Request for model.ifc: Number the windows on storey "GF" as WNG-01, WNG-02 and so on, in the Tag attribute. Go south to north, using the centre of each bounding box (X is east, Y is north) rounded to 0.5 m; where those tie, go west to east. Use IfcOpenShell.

First a look at what the model holds.

```python
import ifcopenshell
import ifcopenshell.util.element
import ifcopenshell.util.placement

model = ifcopenshell.open("model.ifc")
print(model.schema)
storey = next(s for s in model.by_type("IfcBuildingStorey") if s.Name == "GF")
windows = [e for e in ifcopenshell.util.element.get_decomposition(storey) if e.is_a("IfcWindow")]
for e in sorted(windows, key=lambda e: e.id()):
    origin = ifcopenshell.util.placement.get_local_placement(e.ObjectPlacement)[:3, 3]
    print(e.id(), e.Tag, e.Name, origin.round(2) + 0.0, sep=" | ")
```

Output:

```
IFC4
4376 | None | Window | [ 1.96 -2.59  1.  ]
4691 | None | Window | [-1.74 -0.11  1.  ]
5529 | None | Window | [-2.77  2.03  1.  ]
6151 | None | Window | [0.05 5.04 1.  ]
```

```python
import ifcopenshell
import ifcopenshell.geom
import ifcopenshell.util.element
import ifcopenshell.util.shape

model = ifcopenshell.open("model.ifc")
settings = ifcopenshell.geom.settings()
settings.set("use-world-coords", True)


def centre(element):
    shape = ifcopenshell.geom.create_shape(settings, element)
    return ifcopenshell.util.shape.get_bbox_centroid(shape.geometry)


storey = next(s for s in model.by_type("IfcBuildingStorey") if s.Name == "GF")
windows = [e for e in ifcopenshell.util.element.get_decomposition(storey) if e.is_a("IfcWindow")]

# Insertion points can sit at a corner or the storey origin, so sort by the geometry (in metres).
centres = {e: centre(e) for e in windows}
windows.sort(key=lambda e: (round(centres[e][1] / 0.5), centres[e][0]))

for i, e in enumerate(windows, start=1):
    number = f"WNG-{i:02d}"
    e.Tag = number
    print(e.id(), number)

model.write("model_rev.ifc")
```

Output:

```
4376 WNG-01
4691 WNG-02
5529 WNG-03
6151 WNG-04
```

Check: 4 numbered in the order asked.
